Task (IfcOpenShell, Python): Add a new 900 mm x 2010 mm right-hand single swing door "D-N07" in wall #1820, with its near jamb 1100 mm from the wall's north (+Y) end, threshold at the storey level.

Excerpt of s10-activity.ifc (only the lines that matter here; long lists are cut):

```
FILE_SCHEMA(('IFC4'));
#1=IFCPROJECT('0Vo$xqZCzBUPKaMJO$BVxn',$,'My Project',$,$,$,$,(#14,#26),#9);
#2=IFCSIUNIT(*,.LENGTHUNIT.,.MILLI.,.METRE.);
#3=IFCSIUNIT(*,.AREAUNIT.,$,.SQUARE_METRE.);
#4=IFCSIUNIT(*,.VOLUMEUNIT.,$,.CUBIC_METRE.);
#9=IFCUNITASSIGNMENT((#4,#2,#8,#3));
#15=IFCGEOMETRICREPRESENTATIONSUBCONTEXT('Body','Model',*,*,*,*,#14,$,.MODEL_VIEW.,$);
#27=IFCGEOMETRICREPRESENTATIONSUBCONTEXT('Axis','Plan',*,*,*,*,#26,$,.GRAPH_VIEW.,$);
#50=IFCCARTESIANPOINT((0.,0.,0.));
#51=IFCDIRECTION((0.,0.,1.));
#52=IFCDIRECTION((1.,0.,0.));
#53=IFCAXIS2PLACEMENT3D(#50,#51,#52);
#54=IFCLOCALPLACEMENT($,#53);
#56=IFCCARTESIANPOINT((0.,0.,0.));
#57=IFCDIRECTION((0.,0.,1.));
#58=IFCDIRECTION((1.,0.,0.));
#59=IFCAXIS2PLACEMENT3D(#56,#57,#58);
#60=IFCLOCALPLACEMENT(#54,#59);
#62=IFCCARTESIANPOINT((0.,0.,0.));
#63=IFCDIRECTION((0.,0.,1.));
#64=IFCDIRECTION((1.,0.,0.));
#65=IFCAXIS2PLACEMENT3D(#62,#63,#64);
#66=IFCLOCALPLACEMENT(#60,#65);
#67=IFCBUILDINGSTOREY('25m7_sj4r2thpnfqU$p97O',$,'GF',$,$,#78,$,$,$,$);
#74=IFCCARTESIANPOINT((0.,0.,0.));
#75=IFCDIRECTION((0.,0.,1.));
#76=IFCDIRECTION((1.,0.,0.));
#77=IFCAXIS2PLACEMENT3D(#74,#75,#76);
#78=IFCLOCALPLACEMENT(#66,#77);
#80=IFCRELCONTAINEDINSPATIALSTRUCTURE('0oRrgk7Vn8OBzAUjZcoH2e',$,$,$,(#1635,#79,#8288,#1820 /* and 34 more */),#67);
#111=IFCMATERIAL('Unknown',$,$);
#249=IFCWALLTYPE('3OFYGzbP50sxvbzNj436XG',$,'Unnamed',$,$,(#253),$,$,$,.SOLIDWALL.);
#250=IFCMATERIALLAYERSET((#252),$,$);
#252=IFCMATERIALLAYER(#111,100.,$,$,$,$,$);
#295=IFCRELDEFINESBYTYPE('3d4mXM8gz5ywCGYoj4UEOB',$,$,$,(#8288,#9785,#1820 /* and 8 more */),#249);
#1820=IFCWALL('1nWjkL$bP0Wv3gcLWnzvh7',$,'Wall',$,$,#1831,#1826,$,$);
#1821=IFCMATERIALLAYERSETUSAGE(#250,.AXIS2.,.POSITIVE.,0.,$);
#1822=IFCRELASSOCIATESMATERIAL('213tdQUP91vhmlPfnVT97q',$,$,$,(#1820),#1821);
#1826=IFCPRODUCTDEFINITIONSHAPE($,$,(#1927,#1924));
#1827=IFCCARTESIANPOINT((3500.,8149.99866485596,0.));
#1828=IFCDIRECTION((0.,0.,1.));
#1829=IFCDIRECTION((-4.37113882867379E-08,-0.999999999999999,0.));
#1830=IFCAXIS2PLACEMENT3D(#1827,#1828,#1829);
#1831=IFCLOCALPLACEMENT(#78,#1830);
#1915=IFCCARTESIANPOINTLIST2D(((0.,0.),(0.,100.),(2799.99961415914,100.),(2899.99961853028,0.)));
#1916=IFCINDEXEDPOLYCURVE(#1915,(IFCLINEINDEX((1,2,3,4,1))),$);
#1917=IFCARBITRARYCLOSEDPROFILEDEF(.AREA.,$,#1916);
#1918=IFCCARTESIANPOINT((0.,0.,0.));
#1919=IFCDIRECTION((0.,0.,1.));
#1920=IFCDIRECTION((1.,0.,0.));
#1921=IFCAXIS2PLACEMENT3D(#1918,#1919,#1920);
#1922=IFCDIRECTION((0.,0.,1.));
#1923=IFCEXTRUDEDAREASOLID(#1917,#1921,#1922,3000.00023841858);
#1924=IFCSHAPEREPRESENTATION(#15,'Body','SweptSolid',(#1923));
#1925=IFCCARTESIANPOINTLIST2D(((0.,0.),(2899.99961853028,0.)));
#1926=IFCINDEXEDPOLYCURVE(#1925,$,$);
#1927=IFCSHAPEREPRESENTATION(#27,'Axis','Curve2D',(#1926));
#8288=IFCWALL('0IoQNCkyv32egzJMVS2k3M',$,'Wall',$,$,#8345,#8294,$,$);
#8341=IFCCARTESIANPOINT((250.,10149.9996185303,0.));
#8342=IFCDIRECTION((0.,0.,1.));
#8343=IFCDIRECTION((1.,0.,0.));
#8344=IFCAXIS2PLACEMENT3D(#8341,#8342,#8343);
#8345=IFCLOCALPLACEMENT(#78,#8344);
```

```python
import numpy as np
import ifcopenshell
import ifcopenshell.api.feature
import ifcopenshell.api.geometry
import ifcopenshell.api.root
import ifcopenshell.api.spatial
import ifcopenshell.geom
import ifcopenshell.util.element
import ifcopenshell.util.placement
import ifcopenshell.util.representation
import ifcopenshell.util.shape
import ifcopenshell.util.unit

model = ifcopenshell.open("s10-activity.ifc")
unit_scale = ifcopenshell.util.unit.calculate_unit_scale(model)
settings = ifcopenshell.geom.settings()


def volume(element):
    """Net volume in cubic metres, openings subtracted."""
    shape = ifcopenshell.geom.create_shape(settings, element)
    return ifcopenshell.util.shape.get_volume(shape.geometry)


wall = model.by_guid("1nWjkL$bP0Wv3gcLWnzvh7")
storey = ifcopenshell.util.element.get_container(wall, ifc_class="IfcBuildingStorey")
context = ifcopenshell.util.representation.get_context(model, "Model", "Body", "MODEL_VIEW")
before = volume(wall)

width, height, from_end, sill = 0.9, 2.01, 1.1, 0.0  # metres

# The wall runs along its own X axis, and the end named is its -X end.
wall_shape = ifcopenshell.geom.create_shape(settings, wall)
x, y, z = ifcopenshell.util.shape.get_vertices(wall_shape.geometry).T
start = x.min() + from_end
face, thickness = float(y.min()), float(y.max() - y.min())
wall_matrix = ifcopenshell.util.placement.get_local_placement(wall.ObjectPlacement)
level = ifcopenshell.util.placement.get_local_placement(storey.ObjectPlacement)[2, 3]


def in_wall(x, y):
    """Placement at x, y metres in the wall's axes, at sill height."""
    matrix = wall_matrix.copy()
    matrix[:, 3] = wall_matrix @ np.array([x / unit_scale, y / unit_scale, 0.0, 1.0])
    matrix[2, 3] = level + sill / unit_scale
    return matrix


# Opening: a box that overshoots both wall faces by 50 mm.
opening = ifcopenshell.api.root.create_entity(model, ifc_class="IfcOpeningElement", predefined_type="OPENING")
box = ifcopenshell.api.geometry.add_wall_representation(
    model, context=context, length=width, height=height, thickness=thickness + 0.1
)
ifcopenshell.api.geometry.assign_representation(model, product=opening, representation=box)
ifcopenshell.api.geometry.edit_object_placement(model, product=opening, matrix=in_wall(start, face - 0.05), is_si=False)
ifcopenshell.api.feature.add_feature(model, feature=opening, element=wall)

door = ifcopenshell.api.root.create_entity(model, ifc_class="IfcDoor", name="D-N07", predefined_type="DOOR")
door.OverallWidth, door.OverallHeight = width / unit_scale, height / unit_scale
door.OperationType = "SINGLE_SWING_RIGHT"
body = ifcopenshell.api.geometry.add_door_representation(
    model,
    context=context,
    overall_width=door.OverallWidth,
    overall_height=door.OverallHeight,
    operation_type="SINGLE_SWING_RIGHT",
    lining_properties={"LiningDepth": thickness / unit_scale, "ThresholdDepth": thickness / unit_scale},
)
ifcopenshell.api.geometry.assign_representation(model, product=door, representation=body)
ifcopenshell.api.spatial.assign_container(model, products=[door], relating_structure=storey)
ifcopenshell.api.feature.add_filling(model, opening=opening, element=door)

# The lining spans the wall, so the door starts at the wall face.
ifcopenshell.api.geometry.edit_object_placement(model, product=door, matrix=in_wall(start, face), is_si=False)

after = volume(wall)

print(f"wall volume {before:.3f} -> {after:.3f} m3")

model.write("s10-activity_edited.ifc")
```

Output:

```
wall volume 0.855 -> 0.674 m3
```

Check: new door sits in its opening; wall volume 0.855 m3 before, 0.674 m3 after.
